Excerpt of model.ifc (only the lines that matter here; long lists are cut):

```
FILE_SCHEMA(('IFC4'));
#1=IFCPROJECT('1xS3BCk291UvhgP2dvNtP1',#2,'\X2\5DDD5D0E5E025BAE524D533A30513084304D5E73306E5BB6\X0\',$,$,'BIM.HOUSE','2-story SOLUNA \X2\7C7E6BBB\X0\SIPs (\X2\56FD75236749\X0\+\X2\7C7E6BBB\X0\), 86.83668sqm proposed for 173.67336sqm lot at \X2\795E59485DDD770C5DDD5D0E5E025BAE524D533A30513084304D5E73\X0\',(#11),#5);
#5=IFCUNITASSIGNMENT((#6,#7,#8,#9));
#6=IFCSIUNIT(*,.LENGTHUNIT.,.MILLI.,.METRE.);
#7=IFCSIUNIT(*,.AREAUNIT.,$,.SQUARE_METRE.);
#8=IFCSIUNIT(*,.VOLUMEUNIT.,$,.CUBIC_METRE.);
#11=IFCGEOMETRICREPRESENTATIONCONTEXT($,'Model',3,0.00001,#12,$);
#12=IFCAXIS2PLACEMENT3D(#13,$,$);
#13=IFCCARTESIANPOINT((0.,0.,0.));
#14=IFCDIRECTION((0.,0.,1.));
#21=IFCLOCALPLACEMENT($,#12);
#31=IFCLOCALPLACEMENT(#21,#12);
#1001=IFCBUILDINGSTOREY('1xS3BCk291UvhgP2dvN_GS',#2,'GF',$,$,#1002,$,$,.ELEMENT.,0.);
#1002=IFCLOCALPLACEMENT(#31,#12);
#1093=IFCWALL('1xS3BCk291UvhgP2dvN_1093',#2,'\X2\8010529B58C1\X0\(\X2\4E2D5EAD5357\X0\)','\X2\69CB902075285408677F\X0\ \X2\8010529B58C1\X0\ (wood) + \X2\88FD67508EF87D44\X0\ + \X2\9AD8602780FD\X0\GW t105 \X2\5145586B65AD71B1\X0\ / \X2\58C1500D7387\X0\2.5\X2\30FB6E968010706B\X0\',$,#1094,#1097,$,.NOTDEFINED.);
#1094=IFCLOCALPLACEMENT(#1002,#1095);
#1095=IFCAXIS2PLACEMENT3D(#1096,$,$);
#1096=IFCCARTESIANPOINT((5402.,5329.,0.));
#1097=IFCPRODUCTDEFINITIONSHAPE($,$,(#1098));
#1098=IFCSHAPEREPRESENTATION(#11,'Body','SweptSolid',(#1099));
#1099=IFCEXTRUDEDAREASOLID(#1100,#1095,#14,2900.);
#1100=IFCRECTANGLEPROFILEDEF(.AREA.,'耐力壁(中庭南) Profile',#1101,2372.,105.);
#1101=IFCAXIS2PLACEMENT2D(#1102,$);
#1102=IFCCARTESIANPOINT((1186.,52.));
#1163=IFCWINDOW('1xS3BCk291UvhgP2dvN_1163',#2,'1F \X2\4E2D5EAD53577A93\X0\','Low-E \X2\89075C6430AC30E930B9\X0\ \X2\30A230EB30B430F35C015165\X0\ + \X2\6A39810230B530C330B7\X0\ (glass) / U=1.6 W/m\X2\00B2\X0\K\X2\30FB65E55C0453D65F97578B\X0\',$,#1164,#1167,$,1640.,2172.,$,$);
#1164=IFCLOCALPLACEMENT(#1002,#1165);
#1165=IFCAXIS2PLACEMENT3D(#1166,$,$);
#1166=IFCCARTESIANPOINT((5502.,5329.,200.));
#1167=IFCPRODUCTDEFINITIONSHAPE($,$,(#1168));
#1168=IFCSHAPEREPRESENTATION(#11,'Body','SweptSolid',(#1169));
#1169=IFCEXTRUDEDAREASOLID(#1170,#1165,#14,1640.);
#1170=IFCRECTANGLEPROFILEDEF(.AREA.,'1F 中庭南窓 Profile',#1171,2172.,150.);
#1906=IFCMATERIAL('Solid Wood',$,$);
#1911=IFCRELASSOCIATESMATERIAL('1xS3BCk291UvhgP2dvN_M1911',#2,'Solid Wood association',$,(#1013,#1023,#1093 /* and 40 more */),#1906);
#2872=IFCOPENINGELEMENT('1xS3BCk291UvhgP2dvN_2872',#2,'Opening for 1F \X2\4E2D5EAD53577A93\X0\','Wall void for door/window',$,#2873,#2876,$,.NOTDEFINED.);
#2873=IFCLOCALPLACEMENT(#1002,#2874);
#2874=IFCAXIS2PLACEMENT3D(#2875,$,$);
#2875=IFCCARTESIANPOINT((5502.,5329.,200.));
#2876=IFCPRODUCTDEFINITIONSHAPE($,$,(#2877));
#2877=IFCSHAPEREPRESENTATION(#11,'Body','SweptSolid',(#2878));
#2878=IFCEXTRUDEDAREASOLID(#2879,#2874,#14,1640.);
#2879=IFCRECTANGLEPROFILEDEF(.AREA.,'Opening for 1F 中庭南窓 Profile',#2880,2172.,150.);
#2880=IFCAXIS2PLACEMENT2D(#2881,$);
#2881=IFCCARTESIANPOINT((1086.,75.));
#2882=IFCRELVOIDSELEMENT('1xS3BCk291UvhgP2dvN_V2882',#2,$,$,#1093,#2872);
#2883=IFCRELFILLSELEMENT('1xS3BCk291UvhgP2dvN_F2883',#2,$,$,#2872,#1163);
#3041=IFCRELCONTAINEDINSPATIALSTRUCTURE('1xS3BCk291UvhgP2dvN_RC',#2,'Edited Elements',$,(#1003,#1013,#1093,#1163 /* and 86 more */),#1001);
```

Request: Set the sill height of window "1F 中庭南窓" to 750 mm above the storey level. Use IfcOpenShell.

```python
import numpy as np
import ifcopenshell
import ifcopenshell.api.geometry
import ifcopenshell.geom
import ifcopenshell.util.element
import ifcopenshell.util.placement
import ifcopenshell.util.shape
import ifcopenshell.util.unit

model = ifcopenshell.open("model.ifc")
unit_scale = ifcopenshell.util.unit.calculate_unit_scale(model)

window = model.by_guid("1xS3BCk291UvhgP2dvN_1163")
opening = window.FillsVoids[0].RelatingOpeningElement
storey = ifcopenshell.util.element.get_container(window, ifc_class="IfcBuildingStorey")
level = ifcopenshell.util.placement.get_local_placement(storey.ObjectPlacement)[2, 3]

# The opening's origin need not be at the sill, so measure its lowest point.
shape = ifcopenshell.geom.create_shape(ifcopenshell.geom.settings(), opening)
bottom = ifcopenshell.util.shape.get_shape_bottom_elevation(shape, shape.geometry) / unit_scale
dz = level + 750.0 - bottom

shift = np.array([0.0, 0.0, dz])
# The window is not placed relative to its opening, so move both.
for product in (opening, window):
    matrix = ifcopenshell.util.placement.get_local_placement(product.ObjectPlacement)
    matrix[:3, 3] += shift
    ifcopenshell.api.geometry.edit_object_placement(model, product=product, matrix=matrix, is_si=False)

print(f"moved by {dz * unit_scale:+.3f} m")

model.write("model_v2.ifc")
```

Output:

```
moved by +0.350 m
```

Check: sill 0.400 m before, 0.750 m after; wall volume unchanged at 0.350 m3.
